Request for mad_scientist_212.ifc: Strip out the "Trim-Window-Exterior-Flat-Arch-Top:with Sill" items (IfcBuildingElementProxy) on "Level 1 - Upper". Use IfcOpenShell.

First a look at what the model holds.

```python
import ifcopenshell
import ifcopenshell.util.element

model = ifcopenshell.open("mad_scientist_212.ifc")
print(model.schema)
storey = next(s for s in model.by_type("IfcBuildingStorey") if s.Name == "Level 1 - Upper")
proxies = [e for e in ifcopenshell.util.element.get_decomposition(storey) if e.is_a("IfcBuildingElementProxy")]
seen = {}
for e in proxies:
    element_type = ifcopenshell.util.element.get_type(e)
    name = element_type.Name if element_type not in (None, e) else None
    seen[name] = seen.get(name, 0) + 1
for name, count in sorted(seen.items(), key=str):
    print(count, "x", name)
```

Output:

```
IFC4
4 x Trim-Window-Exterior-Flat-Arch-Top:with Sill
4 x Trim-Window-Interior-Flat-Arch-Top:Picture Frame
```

```python
import ifcopenshell
import ifcopenshell.api.root
import ifcopenshell.util.element

model = ifcopenshell.open("mad_scientist_212.ifc")

storey = next(s for s in model.by_type("IfcBuildingStorey") if s.Name == "Level 1 - Upper")
proxies = [e for e in ifcopenshell.util.element.get_decomposition(storey) if e.is_a("IfcBuildingElementProxy")]
targets = [e for e in proxies if (t := ifcopenshell.util.element.get_type(e)) not in (None, e) and t.Name == "Trim-Window-Exterior-Flat-Arch-Top:with Sill"]

for e in targets:
    ifcopenshell.api.root.remove_product(model, product=e)
print(len(targets), "removed")

model.write("mad_scientist_212_updated.ifc")
```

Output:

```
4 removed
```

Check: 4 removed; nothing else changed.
